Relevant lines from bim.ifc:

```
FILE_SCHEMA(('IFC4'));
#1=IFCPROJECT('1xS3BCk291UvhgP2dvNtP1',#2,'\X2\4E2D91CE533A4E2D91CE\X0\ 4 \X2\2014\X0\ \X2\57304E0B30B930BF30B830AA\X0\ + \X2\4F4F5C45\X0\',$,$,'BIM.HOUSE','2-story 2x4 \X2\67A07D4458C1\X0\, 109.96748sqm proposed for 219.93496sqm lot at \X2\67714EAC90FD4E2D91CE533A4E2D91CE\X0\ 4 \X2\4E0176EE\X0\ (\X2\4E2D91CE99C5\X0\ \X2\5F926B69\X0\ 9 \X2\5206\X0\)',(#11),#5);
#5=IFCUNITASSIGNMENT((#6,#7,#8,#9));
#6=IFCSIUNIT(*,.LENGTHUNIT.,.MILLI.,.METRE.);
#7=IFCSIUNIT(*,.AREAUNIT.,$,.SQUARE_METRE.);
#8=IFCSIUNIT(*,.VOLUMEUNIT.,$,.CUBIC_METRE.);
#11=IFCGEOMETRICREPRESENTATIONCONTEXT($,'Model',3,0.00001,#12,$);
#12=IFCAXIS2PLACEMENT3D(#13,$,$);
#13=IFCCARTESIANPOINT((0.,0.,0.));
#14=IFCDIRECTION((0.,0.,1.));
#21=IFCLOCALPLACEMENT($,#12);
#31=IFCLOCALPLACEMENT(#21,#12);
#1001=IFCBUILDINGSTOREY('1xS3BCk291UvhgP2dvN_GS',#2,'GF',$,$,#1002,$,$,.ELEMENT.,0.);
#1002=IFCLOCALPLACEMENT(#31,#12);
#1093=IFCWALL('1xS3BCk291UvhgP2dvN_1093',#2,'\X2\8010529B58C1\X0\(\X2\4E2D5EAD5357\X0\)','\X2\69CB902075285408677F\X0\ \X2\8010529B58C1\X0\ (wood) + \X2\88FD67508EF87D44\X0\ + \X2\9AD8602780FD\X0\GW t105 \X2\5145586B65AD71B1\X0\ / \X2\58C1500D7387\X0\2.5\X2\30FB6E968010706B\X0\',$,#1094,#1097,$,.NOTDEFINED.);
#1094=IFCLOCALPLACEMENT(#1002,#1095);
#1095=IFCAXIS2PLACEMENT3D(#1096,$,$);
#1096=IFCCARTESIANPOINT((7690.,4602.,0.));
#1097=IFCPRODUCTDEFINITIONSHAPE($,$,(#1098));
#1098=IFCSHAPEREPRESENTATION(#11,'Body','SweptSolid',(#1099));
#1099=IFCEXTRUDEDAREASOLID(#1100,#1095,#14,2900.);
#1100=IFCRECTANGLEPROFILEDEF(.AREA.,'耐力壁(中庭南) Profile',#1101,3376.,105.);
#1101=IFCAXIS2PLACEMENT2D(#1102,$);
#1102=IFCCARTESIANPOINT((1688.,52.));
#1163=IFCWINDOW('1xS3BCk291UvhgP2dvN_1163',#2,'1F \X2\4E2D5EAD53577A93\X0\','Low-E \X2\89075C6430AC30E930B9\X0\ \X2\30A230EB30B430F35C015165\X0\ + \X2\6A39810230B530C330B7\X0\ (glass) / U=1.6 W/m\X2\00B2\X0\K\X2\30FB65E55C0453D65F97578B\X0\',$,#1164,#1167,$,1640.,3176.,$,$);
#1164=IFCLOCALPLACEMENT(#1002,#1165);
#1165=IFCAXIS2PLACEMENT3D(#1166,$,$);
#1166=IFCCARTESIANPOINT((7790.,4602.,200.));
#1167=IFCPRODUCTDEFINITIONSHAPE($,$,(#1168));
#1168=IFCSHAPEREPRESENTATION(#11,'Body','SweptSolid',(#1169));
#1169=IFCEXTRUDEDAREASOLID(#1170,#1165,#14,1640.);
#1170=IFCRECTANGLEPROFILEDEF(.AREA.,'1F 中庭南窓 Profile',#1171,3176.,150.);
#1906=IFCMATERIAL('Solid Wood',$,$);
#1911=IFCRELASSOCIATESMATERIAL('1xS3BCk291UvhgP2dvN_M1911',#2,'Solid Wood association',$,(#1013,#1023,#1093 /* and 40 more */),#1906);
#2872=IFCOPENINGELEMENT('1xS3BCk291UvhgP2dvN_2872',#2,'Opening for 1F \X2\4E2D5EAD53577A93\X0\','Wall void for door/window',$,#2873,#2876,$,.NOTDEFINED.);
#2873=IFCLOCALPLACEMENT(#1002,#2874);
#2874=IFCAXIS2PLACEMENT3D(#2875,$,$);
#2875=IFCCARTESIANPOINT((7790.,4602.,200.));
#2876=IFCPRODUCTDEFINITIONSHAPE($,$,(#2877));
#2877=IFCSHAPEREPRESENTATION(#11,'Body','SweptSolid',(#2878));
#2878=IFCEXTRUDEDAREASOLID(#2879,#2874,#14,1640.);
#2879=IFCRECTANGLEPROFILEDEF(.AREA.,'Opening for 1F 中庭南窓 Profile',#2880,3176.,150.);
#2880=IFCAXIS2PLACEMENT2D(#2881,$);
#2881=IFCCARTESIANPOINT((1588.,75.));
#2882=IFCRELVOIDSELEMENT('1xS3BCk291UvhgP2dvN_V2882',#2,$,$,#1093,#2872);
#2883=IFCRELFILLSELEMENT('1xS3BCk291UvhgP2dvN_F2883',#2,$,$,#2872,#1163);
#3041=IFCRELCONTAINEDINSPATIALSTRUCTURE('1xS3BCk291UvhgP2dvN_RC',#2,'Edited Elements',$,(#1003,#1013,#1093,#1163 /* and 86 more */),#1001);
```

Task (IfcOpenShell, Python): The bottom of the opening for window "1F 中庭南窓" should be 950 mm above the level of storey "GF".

```python
import numpy as np
import ifcopenshell
import ifcopenshell.api.geometry
import ifcopenshell.geom
import ifcopenshell.util.element
import ifcopenshell.util.placement
import ifcopenshell.util.shape
import ifcopenshell.util.unit

model = ifcopenshell.open("bim.ifc")
unit_scale = ifcopenshell.util.unit.calculate_unit_scale(model)

window = model.by_id(1163)
opening = window.FillsVoids[0].RelatingOpeningElement
storey = ifcopenshell.util.element.get_container(window, ifc_class="IfcBuildingStorey")
level = ifcopenshell.util.placement.get_local_placement(storey.ObjectPlacement)[2, 3]

# The opening's origin need not be at the sill, so measure its lowest point.
shape = ifcopenshell.geom.create_shape(ifcopenshell.geom.settings(), opening)
bottom = ifcopenshell.util.shape.get_shape_bottom_elevation(shape, shape.geometry) / unit_scale
dz = level + 950.0 - bottom

shift = np.array([0.0, 0.0, dz])
# The window is not placed relative to its opening, so move both.
for product in (opening, window):
    matrix = ifcopenshell.util.placement.get_local_placement(product.ObjectPlacement)
    matrix[:3, 3] += shift
    ifcopenshell.api.geometry.edit_object_placement(model, product=product, matrix=matrix, is_si=False)

print(f"moved by {dz * unit_scale:+.3f} m")

model.write("bim_rev.ifc")
```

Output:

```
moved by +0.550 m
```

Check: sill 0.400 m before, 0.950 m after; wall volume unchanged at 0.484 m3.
